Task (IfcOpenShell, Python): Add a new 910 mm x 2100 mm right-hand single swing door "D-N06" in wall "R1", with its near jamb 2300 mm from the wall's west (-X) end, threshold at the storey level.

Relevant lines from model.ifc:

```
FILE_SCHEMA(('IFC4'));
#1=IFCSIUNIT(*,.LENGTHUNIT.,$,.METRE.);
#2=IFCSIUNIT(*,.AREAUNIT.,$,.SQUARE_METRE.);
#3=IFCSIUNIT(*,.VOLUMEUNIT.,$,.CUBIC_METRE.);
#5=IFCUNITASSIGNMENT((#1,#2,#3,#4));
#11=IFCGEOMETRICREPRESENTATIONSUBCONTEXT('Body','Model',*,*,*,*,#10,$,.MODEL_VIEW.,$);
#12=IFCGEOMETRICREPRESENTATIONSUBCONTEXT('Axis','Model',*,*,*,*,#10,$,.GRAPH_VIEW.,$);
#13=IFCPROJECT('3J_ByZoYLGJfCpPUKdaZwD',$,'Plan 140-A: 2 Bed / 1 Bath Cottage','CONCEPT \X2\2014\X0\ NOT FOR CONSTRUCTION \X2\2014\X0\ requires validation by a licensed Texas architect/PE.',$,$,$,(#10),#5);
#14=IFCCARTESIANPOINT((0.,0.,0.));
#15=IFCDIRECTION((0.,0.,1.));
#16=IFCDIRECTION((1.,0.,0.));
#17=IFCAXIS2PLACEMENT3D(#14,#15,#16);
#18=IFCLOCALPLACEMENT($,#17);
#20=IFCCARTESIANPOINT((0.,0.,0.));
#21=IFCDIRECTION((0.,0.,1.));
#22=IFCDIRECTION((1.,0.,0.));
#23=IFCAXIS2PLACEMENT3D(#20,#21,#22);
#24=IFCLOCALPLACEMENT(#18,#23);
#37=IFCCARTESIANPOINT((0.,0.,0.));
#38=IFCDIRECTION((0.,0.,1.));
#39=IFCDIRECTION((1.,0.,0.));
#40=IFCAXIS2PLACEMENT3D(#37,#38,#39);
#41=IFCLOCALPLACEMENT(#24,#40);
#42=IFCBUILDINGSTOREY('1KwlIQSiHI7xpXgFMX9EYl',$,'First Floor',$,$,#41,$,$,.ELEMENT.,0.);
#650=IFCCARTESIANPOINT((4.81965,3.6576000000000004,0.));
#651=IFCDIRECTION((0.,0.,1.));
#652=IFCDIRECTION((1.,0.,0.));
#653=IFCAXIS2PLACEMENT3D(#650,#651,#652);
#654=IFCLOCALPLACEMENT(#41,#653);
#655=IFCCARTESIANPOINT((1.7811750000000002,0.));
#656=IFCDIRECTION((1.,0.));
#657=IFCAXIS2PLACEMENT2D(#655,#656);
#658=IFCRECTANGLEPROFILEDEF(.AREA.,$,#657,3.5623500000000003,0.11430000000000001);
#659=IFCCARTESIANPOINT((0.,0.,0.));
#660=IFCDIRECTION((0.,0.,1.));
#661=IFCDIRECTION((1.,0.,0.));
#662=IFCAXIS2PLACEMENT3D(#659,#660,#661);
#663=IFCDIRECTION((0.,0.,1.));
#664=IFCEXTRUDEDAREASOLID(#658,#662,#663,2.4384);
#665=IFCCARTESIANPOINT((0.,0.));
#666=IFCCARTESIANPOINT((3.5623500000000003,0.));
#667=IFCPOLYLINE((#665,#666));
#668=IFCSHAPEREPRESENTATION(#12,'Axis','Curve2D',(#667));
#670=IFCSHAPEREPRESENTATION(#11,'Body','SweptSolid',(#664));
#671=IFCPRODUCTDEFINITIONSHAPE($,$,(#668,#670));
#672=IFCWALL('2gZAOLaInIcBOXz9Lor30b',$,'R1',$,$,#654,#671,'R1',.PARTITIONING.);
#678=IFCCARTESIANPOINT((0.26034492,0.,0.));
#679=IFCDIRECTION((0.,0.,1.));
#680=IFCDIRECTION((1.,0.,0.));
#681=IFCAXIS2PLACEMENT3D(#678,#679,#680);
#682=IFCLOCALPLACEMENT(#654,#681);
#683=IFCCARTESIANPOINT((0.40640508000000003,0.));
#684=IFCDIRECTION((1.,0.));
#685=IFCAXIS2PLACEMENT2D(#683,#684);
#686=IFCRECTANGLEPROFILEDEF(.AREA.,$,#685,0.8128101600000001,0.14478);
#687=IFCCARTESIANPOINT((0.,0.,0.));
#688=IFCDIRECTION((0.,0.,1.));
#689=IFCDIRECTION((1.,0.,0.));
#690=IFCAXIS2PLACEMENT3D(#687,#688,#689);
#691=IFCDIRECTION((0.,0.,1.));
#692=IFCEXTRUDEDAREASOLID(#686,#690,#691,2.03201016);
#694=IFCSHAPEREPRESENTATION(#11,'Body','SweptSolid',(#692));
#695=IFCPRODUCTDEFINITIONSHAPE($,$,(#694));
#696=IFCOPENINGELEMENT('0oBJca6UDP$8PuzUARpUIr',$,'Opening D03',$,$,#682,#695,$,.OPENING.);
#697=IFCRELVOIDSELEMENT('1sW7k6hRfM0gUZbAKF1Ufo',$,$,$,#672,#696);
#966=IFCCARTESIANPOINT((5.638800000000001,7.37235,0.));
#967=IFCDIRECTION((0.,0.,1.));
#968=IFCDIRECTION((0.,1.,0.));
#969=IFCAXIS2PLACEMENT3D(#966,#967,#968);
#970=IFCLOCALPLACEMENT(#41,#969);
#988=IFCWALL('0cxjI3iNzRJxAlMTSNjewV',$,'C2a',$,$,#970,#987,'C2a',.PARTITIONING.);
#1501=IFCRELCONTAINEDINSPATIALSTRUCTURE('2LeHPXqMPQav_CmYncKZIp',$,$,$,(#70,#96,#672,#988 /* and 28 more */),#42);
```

```python
import numpy as np
import ifcopenshell
import ifcopenshell.api.feature
import ifcopenshell.api.geometry
import ifcopenshell.api.root
import ifcopenshell.api.spatial
import ifcopenshell.geom
import ifcopenshell.util.element
import ifcopenshell.util.placement
import ifcopenshell.util.representation
import ifcopenshell.util.shape
import ifcopenshell.util.unit

model = ifcopenshell.open("model.ifc")
unit_scale = ifcopenshell.util.unit.calculate_unit_scale(model)
settings = ifcopenshell.geom.settings()


def volume(element):
    """Net volume in cubic metres, openings subtracted."""
    shape = ifcopenshell.geom.create_shape(settings, element)
    return ifcopenshell.util.shape.get_volume(shape.geometry)


wall = model.by_guid("2gZAOLaInIcBOXz9Lor30b")
storey = ifcopenshell.util.element.get_container(wall, ifc_class="IfcBuildingStorey")
context = ifcopenshell.util.representation.get_context(model, "Model", "Body", "MODEL_VIEW")
before = volume(wall)

width, height, from_end, sill = 0.91, 2.1, 2.3, 0.0  # metres

# The wall runs along its own X axis, and the end named is its -X end.
wall_shape = ifcopenshell.geom.create_shape(settings, wall)
x, y, z = ifcopenshell.util.shape.get_vertices(wall_shape.geometry).T
start = x.min() + from_end
face, thickness = float(y.min()), float(y.max() - y.min())
wall_matrix = ifcopenshell.util.placement.get_local_placement(wall.ObjectPlacement)
level = ifcopenshell.util.placement.get_local_placement(storey.ObjectPlacement)[2, 3]


def in_wall(x, y):
    """Placement at x, y metres in the wall's axes, at sill height."""
    matrix = wall_matrix.copy()
    matrix[:, 3] = wall_matrix @ np.array([x / unit_scale, y / unit_scale, 0.0, 1.0])
    matrix[2, 3] = level + sill / unit_scale
    return matrix


# Opening: a box that overshoots both wall faces by 50 mm.
opening = ifcopenshell.api.root.create_entity(model, ifc_class="IfcOpeningElement", predefined_type="OPENING")
box = ifcopenshell.api.geometry.add_wall_representation(
    model, context=context, length=width, height=height, thickness=thickness + 0.1
)
ifcopenshell.api.geometry.assign_representation(model, product=opening, representation=box)
ifcopenshell.api.geometry.edit_object_placement(model, product=opening, matrix=in_wall(start, face - 0.05), is_si=False)
ifcopenshell.api.feature.add_feature(model, feature=opening, element=wall)

door = ifcopenshell.api.root.create_entity(model, ifc_class="IfcDoor", name="D-N06", predefined_type="DOOR")
door.OverallWidth, door.OverallHeight = width / unit_scale, height / unit_scale
door.OperationType = "SINGLE_SWING_RIGHT"
body = ifcopenshell.api.geometry.add_door_representation(
    model,
    context=context,
    overall_width=door.OverallWidth,
    overall_height=door.OverallHeight,
    operation_type="SINGLE_SWING_RIGHT",
    lining_properties={"LiningDepth": thickness / unit_scale, "ThresholdDepth": thickness / unit_scale},
)
ifcopenshell.api.geometry.assign_representation(model, product=door, representation=body)
ifcopenshell.api.spatial.assign_container(model, products=[door], relating_structure=storey)
ifcopenshell.api.feature.add_filling(model, opening=opening, element=door)

# The lining spans the wall, so the door starts at the wall face.
ifcopenshell.api.geometry.edit_object_placement(model, product=door, matrix=in_wall(start, face), is_si=False)

after = volume(wall)

print(f"wall volume {before:.3f} -> {after:.3f} m3")

model.write("model_updated.ifc")
```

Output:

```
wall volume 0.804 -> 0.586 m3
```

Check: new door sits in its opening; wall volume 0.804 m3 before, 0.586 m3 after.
